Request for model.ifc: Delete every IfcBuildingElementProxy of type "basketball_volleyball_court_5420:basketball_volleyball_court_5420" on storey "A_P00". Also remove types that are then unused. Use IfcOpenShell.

First a look at what the model holds.

```python
import ifcopenshell
import ifcopenshell.util.element

model = ifcopenshell.open("model.ifc")
print(model.schema)
storey = next(s for s in model.by_type("IfcBuildingStorey") if s.Name == "A_P00")
proxies = [e for e in ifcopenshell.util.element.get_decomposition(storey) if e.is_a("IfcBuildingElementProxy")]
seen = {}
for e in proxies:
    element_type = ifcopenshell.util.element.get_type(e)
    name = element_type.Name if element_type not in (None, e) else None
    seen[name] = seen.get(name, 0) + 1
for name, count in sorted(seen.items(), key=str):
    print(count, "x", name)
```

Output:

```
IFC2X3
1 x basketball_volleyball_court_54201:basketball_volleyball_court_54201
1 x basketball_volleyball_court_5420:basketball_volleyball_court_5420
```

```python
import ifcopenshell
import ifcopenshell.api.root
import ifcopenshell.util.element

model = ifcopenshell.open("model.ifc")

storey = next(s for s in model.by_type("IfcBuildingStorey") if s.Name == "A_P00")
proxies = [e for e in ifcopenshell.util.element.get_decomposition(storey) if e.is_a("IfcBuildingElementProxy")]
targets = [e for e in proxies if (t := ifcopenshell.util.element.get_type(e)) not in (None, e) and t.Name == "basketball_volleyball_court_5420:basketball_volleyball_court_5420"]
types = {ifcopenshell.util.element.get_type(e) for e in targets} - {None, *targets}

for e in targets:
    ifcopenshell.api.root.remove_product(model, product=e)
print(len(targets), "removed")

unused = [t for t in types if not ifcopenshell.util.element.get_types(t)]
for t in unused:
    ifcopenshell.api.root.remove_product(model, product=t)
print(len(unused), "unused types removed")

model.write("model_v2.ifc")
```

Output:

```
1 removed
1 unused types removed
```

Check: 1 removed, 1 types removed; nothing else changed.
